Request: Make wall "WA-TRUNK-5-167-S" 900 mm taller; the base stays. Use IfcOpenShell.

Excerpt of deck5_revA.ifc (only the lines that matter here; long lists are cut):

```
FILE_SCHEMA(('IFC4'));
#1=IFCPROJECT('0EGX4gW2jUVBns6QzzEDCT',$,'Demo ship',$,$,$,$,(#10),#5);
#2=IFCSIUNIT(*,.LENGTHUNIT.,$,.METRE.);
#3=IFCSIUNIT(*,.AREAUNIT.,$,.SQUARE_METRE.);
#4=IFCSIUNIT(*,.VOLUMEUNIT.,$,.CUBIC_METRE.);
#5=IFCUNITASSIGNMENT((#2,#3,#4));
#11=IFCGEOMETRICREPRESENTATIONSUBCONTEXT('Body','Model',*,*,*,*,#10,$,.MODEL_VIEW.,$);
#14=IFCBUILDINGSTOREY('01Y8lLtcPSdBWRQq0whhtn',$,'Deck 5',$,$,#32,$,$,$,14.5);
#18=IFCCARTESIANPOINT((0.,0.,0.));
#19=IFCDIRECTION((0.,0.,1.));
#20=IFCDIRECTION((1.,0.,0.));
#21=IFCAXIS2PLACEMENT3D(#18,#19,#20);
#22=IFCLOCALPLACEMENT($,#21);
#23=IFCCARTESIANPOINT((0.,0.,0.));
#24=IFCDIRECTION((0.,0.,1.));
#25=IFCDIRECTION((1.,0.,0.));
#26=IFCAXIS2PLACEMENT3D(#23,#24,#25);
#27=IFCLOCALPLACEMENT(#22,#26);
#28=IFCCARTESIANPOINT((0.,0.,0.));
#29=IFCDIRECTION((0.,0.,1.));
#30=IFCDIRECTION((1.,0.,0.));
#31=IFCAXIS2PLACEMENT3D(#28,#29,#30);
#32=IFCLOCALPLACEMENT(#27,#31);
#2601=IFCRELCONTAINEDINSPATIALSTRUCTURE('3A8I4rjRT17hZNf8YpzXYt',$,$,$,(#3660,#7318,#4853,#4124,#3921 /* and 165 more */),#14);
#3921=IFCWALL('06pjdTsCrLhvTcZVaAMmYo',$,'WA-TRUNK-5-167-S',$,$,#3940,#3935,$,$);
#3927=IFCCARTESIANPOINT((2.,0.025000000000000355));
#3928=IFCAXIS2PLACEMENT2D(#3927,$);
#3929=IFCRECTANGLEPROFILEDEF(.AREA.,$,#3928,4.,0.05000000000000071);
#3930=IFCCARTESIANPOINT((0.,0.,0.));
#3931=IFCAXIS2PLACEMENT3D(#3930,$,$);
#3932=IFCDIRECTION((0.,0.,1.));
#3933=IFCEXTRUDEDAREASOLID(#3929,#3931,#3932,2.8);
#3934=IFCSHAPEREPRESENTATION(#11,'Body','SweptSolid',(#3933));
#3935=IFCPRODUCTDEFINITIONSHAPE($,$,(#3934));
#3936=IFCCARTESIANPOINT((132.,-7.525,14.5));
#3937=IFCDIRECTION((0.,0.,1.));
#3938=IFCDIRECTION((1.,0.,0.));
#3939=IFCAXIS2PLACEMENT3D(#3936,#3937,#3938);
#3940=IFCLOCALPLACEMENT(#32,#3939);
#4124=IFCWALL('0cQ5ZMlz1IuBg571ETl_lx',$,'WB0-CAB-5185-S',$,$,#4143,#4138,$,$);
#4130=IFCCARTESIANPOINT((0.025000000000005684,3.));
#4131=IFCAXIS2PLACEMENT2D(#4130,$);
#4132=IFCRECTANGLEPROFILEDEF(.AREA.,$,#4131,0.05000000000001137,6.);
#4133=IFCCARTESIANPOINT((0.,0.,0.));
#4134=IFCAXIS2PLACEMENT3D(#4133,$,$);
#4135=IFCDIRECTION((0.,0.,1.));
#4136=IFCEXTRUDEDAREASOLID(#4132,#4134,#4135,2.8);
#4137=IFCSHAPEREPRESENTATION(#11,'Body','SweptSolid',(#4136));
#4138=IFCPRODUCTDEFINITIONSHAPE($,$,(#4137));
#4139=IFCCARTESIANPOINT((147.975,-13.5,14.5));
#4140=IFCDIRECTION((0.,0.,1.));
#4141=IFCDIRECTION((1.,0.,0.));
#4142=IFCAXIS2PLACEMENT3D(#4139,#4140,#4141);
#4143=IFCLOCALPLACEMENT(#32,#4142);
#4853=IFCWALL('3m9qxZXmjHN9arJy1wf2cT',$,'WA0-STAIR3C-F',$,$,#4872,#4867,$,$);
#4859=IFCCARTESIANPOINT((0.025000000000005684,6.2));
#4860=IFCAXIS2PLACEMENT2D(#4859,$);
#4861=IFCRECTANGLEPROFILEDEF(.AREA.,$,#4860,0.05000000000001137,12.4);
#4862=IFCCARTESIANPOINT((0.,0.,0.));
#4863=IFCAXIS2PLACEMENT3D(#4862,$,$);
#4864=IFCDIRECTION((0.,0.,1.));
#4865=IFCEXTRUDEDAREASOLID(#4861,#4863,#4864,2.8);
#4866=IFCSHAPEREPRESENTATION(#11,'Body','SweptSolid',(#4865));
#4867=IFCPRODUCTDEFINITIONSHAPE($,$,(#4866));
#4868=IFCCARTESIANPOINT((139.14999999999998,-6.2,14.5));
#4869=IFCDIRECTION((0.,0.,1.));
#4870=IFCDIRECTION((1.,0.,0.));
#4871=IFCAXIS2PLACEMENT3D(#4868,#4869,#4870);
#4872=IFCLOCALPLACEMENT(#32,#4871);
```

```python
import ifcopenshell
import ifcopenshell.geom
import ifcopenshell.util.representation
import ifcopenshell.util.shape
import ifcopenshell.util.unit

model = ifcopenshell.open("deck5_revA.ifc")
unit_scale = ifcopenshell.util.unit.calculate_unit_scale(model)
settings = ifcopenshell.geom.settings()


def volume(element):
    """Net volume in cubic metres, openings subtracted."""
    shape = ifcopenshell.geom.create_shape(settings, element)
    return ifcopenshell.util.shape.get_volume(shape.geometry)


wall = model.by_guid("06pjdTsCrLhvTcZVaAMmYo")
before = volume(wall)

body = ifcopenshell.util.representation.get_representation(wall, "Model", "Body")
solid = body.Items[0]
old_height = solid.Depth
solid.Depth += 0.9 / unit_scale
after = volume(wall)

print(f"height {old_height:g} -> {solid.Depth:g}, volume {before:.3f} -> {after:.3f} m3")

model.write("deck5_revA_v2.ifc")
```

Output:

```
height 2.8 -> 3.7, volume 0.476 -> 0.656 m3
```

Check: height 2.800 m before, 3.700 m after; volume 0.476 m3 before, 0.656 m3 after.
